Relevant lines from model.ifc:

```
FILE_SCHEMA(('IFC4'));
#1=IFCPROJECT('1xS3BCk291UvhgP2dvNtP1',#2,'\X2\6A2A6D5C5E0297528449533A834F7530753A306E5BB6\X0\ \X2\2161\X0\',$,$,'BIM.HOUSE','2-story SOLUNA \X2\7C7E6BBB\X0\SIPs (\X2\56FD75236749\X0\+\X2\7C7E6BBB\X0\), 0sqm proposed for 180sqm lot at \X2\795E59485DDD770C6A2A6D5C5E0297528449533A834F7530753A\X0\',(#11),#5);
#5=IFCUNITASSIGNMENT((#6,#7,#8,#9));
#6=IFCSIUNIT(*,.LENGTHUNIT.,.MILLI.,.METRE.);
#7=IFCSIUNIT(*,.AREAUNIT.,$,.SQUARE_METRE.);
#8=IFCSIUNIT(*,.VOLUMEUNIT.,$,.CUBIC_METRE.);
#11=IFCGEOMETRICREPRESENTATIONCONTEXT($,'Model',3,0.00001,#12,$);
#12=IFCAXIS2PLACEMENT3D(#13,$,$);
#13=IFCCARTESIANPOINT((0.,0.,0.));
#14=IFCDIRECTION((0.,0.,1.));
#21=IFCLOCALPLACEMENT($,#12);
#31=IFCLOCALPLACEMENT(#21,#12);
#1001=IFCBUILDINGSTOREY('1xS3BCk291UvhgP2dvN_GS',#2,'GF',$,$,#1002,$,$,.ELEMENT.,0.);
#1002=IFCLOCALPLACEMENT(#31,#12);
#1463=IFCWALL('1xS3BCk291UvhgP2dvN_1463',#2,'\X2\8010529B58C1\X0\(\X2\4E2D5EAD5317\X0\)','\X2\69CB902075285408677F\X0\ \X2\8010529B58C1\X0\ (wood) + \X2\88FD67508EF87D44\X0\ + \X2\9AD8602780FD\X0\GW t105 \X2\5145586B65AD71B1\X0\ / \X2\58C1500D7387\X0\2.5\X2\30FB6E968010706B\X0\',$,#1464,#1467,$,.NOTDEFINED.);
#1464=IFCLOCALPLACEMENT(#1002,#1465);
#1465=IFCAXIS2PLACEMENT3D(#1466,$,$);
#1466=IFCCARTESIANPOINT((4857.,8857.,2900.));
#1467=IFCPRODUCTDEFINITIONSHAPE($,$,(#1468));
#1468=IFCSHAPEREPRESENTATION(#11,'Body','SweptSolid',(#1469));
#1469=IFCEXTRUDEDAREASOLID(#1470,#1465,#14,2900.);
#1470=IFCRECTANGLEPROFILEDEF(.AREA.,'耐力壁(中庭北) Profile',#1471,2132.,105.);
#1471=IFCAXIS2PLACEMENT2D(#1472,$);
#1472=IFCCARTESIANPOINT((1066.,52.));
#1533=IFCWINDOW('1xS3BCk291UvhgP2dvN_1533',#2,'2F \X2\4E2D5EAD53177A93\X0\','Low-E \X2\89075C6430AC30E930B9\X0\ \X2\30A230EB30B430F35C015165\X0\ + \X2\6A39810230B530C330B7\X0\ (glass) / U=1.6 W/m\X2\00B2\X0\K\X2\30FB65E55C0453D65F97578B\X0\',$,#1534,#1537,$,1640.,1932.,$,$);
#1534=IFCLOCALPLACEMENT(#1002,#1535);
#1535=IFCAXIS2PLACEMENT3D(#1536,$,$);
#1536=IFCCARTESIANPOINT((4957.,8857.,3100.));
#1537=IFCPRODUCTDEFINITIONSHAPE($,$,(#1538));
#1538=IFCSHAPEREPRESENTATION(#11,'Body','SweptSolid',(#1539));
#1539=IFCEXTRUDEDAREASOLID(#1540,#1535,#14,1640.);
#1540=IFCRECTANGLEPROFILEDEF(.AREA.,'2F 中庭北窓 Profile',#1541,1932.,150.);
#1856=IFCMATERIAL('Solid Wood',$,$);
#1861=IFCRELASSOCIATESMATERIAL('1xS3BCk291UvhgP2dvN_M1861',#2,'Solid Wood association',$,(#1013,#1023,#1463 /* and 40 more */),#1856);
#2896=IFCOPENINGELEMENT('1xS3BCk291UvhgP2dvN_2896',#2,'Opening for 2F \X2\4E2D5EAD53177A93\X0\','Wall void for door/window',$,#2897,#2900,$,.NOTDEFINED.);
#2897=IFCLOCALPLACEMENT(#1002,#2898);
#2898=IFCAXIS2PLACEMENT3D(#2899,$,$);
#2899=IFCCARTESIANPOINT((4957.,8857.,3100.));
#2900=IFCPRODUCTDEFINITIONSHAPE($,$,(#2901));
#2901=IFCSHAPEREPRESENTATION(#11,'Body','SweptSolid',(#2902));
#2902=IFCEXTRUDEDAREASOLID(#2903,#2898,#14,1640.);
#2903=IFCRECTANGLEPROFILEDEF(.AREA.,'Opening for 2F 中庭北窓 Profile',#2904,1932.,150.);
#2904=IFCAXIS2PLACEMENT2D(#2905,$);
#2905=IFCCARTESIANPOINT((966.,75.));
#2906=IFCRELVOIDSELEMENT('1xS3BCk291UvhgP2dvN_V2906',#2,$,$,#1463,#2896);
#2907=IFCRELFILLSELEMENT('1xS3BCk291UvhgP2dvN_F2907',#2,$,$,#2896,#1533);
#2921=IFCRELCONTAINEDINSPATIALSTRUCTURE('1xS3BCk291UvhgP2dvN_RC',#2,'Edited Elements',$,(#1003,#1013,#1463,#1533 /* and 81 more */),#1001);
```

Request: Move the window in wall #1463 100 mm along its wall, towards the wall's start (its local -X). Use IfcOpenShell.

```python
import ifcopenshell
import ifcopenshell.api.geometry
import ifcopenshell.util.placement

model = ifcopenshell.open("model.ifc")

window = model.by_guid("1xS3BCk291UvhgP2dvN_1533")
opening = window.FillsVoids[0].RelatingOpeningElement
wall = opening.VoidsElements[0].RelatingBuildingElement

wall_matrix = ifcopenshell.util.placement.get_local_placement(wall.ObjectPlacement)
shift = wall_matrix[:3, 0] * -100.0
before = ifcopenshell.util.placement.get_local_placement(window.ObjectPlacement)[:3, 3].copy()

# The window is not placed relative to its opening, so move both.
for product in (opening, window):
    matrix = ifcopenshell.util.placement.get_local_placement(product.ObjectPlacement)
    matrix[:3, 3] += shift
    ifcopenshell.api.geometry.edit_object_placement(model, product=product, matrix=matrix, is_si=False)

after = ifcopenshell.util.placement.get_local_placement(window.ObjectPlacement)[:3, 3]
print("window moved by", (after - before).round(3) + 0.0)

model.write("model_edited.ifc")
```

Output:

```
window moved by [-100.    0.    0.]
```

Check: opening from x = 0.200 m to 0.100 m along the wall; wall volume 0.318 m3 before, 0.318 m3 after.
